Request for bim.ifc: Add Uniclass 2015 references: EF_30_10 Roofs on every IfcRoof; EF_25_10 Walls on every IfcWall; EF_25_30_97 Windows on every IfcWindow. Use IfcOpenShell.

First a look at what the model holds.

```python
import ifcopenshell

model = ifcopenshell.open("bim.ifc")
print(model.schema)
print("classifications:", [c.Name for c in model.by_type("IfcClassification")])
for ifc_class in ("IfcDoor", "IfcRoof", "IfcStair", "IfcWall", "IfcWindow"):
    print(ifc_class, len(model.by_type(ifc_class)))
```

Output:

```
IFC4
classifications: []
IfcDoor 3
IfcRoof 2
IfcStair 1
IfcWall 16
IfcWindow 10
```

```python
import ifcopenshell
import ifcopenshell.api.classification

model = ifcopenshell.open("bim.ifc")

system = ifcopenshell.api.classification.add_classification(model, classification="Uniclass 2015")

codes = {
    "IfcRoof": ("EF_30_10", "Roofs"),
    "IfcWall": ("EF_25_10", "Walls"),
    "IfcWindow": ("EF_25_30_97", "Windows"),
}
for ifc_class, (code, name) in codes.items():
    products = model.by_type(ifc_class)
    ifcopenshell.api.classification.add_reference(
        model, products=products, classification=system, identification=code, name=name
    )
    print(code, len(products))

model.write("bim_updated.ifc")
```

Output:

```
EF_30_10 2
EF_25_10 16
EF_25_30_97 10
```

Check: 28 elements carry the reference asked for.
